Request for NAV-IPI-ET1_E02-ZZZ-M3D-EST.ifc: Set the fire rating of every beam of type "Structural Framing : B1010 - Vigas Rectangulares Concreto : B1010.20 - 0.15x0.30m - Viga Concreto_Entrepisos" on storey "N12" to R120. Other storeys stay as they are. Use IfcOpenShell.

First a look at what the model holds.

```python
import ifcopenshell
import ifcopenshell.util.element

model = ifcopenshell.open("NAV-IPI-ET1_E02-ZZZ-M3D-EST.ifc")
print(model.schema)
storey = next(s for s in model.by_type("IfcBuildingStorey") if s.Name == "N12")
beams = [e for e in ifcopenshell.util.element.get_decomposition(storey) if e.is_a("IfcBeam")]
seen = {}
for e in beams:
    element_type = ifcopenshell.util.element.get_type(e)
    key = (element_type.Name if element_type != e and element_type else None, ifcopenshell.util.element.get_pset(e, "Pset_BeamCommon", "FireRating"))
    seen[key] = seen.get(key, 0) + 1
for (name, value), count in sorted(seen.items(), key=str):
    print(count, "x", name, "|", value)
```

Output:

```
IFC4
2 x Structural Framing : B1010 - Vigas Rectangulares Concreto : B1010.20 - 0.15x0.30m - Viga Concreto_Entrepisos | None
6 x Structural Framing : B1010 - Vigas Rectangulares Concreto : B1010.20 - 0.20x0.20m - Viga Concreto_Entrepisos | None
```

```python
import ifcopenshell
import ifcopenshell.api.pset
import ifcopenshell.util.element

model = ifcopenshell.open("NAV-IPI-ET1_E02-ZZZ-M3D-EST.ifc")

storey = next(s for s in model.by_type("IfcBuildingStorey") if s.Name == "N12")
beams = [e for e in ifcopenshell.util.element.get_decomposition(storey) if e.is_a("IfcBeam")]

count = 0
for e in beams:
    element_type = ifcopenshell.util.element.get_type(e)
    if element_type in (None, e) or element_type.Name != "Structural Framing : B1010 - Vigas Rectangulares Concreto : B1010.20 - 0.15x0.30m - Viga Concreto_Entrepisos":
        continue
    # add_pset returns the element's existing set when there is one.
    pset = ifcopenshell.api.pset.add_pset(model, product=e, name="Pset_BeamCommon")
    ifcopenshell.api.pset.edit_pset(model, pset=pset, properties={"FireRating": "R120"})
    count += 1

print(count, "beams updated")

model.write("NAV-IPI-ET1_E02-ZZZ-M3D-EST_v2.ifc")
```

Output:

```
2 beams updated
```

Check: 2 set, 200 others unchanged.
